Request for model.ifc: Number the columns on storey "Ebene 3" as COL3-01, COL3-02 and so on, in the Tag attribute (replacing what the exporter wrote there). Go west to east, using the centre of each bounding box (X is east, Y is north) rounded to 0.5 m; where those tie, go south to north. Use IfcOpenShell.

First a look at what the model holds.

```python
import ifcopenshell
import ifcopenshell.util.element
import ifcopenshell.util.placement

model = ifcopenshell.open("model.ifc")
print(model.schema)
storey = next(s for s in model.by_type("IfcBuildingStorey") if s.Name == "Ebene 3")
columns = [e for e in ifcopenshell.util.element.get_decomposition(storey) if e.is_a("IfcColumn")]
for e in sorted(columns, key=lambda e: e.id()):
    origin = ifcopenshell.util.placement.get_local_placement(e.ObjectPlacement)[:3, 3]
    print(e.id(), e.Tag, e.Name, origin.round(2) + 0.0, sep=" | ")
```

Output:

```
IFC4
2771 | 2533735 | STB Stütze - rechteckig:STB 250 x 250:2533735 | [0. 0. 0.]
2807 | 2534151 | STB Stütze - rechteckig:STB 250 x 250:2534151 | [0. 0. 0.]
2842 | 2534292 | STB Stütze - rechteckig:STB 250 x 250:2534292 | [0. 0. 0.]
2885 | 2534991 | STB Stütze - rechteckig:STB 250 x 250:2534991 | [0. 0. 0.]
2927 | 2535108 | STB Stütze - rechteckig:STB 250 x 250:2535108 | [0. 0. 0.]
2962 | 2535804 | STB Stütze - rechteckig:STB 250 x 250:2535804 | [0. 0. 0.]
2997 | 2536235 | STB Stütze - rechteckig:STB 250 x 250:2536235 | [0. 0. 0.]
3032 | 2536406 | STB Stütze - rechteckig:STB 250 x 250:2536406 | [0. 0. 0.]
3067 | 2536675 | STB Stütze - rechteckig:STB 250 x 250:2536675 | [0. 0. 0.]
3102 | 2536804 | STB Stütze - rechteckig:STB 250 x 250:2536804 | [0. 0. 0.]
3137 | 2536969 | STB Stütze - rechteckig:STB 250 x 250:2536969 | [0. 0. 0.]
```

```python
import ifcopenshell
import ifcopenshell.geom
import ifcopenshell.util.element
import ifcopenshell.util.shape

model = ifcopenshell.open("model.ifc")
settings = ifcopenshell.geom.settings()
settings.set("use-world-coords", True)


def centre(element):
    shape = ifcopenshell.geom.create_shape(settings, element)
    return ifcopenshell.util.shape.get_bbox_centroid(shape.geometry)


storey = next(s for s in model.by_type("IfcBuildingStorey") if s.Name == "Ebene 3")
columns = [e for e in ifcopenshell.util.element.get_decomposition(storey) if e.is_a("IfcColumn")]

# Insertion points can sit at a corner or the storey origin, so sort by the geometry (in metres).
centres = {e: centre(e) for e in columns}
columns.sort(key=lambda e: (round(centres[e][0] / 0.5), centres[e][1]))

for i, e in enumerate(columns, start=1):
    number = f"COL3-{i:02d}"
    e.Tag = number
    print(e.id(), number)

model.write("model_v2.ifc")
```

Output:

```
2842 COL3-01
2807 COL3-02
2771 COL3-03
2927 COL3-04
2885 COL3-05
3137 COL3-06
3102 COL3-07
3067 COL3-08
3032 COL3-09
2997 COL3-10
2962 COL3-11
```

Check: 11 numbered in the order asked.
